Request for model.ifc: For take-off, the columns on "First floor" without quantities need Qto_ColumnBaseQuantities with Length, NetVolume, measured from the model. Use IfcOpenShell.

First a look at what the model holds.

```python
import ifcopenshell
import ifcopenshell.util.element
import ifcopenshell.util.unit

model = ifcopenshell.open("model.ifc")
print(model.schema)
for unit_type in ("LENGTHUNIT", "AREAUNIT", "VOLUMEUNIT"):
    print(unit_type, ifcopenshell.util.unit.calculate_unit_scale(model, unit_type))
storey = next(s for s in model.by_type("IfcBuildingStorey") if s.Name == "First floor")
columns = [e for e in ifcopenshell.util.element.get_decomposition(storey) if e.is_a("IfcColumn")]
for e in sorted(columns, key=lambda e: e.id()):
    print(e.id(), e.is_a(), e.Name, list(ifcopenshell.util.element.get_psets(e, qtos_only=True)), sep=" | ")
```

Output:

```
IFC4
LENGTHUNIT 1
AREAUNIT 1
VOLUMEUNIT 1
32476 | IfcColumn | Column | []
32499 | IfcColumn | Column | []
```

```python
import ifcopenshell
import ifcopenshell.api.pset
import ifcopenshell.geom
import ifcopenshell.util.element
import ifcopenshell.util.shape
import ifcopenshell.util.unit

model = ifcopenshell.open("model.ifc")
unit_scale = ifcopenshell.util.unit.calculate_unit_scale(model)
volume_scale = ifcopenshell.util.unit.calculate_unit_scale(model, "VOLUMEUNIT")
settings = ifcopenshell.geom.settings()

storey = next(s for s in model.by_type("IfcBuildingStorey") if s.Name == "First floor")
columns = [e for e in ifcopenshell.util.element.get_decomposition(storey) if e.is_a("IfcColumn")]

for e in sorted(columns, key=lambda e: e.id()):
    if ifcopenshell.util.element.get_psets(e, qtos_only=True, should_inherit=False):
        continue
    # Geometry comes back in metres, in the element's own axes.
    shape = ifcopenshell.geom.create_shape(settings, e)
    values = {
        "Length": ifcopenshell.util.shape.get_z(shape.geometry) / unit_scale,
        "NetVolume": ifcopenshell.util.shape.get_volume(shape.geometry) / volume_scale,
    }
    qto = ifcopenshell.api.pset.add_qto(model, product=e, name="Qto_ColumnBaseQuantities")
    ifcopenshell.api.pset.edit_qto(model, qto=qto, properties=values)
    print(e.id(), {k: round(v, 3) for k, v in values.items()})

model.write("model-out.ifc")
```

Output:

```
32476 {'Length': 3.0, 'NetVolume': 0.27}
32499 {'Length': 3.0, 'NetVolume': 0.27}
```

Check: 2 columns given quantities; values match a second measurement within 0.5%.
